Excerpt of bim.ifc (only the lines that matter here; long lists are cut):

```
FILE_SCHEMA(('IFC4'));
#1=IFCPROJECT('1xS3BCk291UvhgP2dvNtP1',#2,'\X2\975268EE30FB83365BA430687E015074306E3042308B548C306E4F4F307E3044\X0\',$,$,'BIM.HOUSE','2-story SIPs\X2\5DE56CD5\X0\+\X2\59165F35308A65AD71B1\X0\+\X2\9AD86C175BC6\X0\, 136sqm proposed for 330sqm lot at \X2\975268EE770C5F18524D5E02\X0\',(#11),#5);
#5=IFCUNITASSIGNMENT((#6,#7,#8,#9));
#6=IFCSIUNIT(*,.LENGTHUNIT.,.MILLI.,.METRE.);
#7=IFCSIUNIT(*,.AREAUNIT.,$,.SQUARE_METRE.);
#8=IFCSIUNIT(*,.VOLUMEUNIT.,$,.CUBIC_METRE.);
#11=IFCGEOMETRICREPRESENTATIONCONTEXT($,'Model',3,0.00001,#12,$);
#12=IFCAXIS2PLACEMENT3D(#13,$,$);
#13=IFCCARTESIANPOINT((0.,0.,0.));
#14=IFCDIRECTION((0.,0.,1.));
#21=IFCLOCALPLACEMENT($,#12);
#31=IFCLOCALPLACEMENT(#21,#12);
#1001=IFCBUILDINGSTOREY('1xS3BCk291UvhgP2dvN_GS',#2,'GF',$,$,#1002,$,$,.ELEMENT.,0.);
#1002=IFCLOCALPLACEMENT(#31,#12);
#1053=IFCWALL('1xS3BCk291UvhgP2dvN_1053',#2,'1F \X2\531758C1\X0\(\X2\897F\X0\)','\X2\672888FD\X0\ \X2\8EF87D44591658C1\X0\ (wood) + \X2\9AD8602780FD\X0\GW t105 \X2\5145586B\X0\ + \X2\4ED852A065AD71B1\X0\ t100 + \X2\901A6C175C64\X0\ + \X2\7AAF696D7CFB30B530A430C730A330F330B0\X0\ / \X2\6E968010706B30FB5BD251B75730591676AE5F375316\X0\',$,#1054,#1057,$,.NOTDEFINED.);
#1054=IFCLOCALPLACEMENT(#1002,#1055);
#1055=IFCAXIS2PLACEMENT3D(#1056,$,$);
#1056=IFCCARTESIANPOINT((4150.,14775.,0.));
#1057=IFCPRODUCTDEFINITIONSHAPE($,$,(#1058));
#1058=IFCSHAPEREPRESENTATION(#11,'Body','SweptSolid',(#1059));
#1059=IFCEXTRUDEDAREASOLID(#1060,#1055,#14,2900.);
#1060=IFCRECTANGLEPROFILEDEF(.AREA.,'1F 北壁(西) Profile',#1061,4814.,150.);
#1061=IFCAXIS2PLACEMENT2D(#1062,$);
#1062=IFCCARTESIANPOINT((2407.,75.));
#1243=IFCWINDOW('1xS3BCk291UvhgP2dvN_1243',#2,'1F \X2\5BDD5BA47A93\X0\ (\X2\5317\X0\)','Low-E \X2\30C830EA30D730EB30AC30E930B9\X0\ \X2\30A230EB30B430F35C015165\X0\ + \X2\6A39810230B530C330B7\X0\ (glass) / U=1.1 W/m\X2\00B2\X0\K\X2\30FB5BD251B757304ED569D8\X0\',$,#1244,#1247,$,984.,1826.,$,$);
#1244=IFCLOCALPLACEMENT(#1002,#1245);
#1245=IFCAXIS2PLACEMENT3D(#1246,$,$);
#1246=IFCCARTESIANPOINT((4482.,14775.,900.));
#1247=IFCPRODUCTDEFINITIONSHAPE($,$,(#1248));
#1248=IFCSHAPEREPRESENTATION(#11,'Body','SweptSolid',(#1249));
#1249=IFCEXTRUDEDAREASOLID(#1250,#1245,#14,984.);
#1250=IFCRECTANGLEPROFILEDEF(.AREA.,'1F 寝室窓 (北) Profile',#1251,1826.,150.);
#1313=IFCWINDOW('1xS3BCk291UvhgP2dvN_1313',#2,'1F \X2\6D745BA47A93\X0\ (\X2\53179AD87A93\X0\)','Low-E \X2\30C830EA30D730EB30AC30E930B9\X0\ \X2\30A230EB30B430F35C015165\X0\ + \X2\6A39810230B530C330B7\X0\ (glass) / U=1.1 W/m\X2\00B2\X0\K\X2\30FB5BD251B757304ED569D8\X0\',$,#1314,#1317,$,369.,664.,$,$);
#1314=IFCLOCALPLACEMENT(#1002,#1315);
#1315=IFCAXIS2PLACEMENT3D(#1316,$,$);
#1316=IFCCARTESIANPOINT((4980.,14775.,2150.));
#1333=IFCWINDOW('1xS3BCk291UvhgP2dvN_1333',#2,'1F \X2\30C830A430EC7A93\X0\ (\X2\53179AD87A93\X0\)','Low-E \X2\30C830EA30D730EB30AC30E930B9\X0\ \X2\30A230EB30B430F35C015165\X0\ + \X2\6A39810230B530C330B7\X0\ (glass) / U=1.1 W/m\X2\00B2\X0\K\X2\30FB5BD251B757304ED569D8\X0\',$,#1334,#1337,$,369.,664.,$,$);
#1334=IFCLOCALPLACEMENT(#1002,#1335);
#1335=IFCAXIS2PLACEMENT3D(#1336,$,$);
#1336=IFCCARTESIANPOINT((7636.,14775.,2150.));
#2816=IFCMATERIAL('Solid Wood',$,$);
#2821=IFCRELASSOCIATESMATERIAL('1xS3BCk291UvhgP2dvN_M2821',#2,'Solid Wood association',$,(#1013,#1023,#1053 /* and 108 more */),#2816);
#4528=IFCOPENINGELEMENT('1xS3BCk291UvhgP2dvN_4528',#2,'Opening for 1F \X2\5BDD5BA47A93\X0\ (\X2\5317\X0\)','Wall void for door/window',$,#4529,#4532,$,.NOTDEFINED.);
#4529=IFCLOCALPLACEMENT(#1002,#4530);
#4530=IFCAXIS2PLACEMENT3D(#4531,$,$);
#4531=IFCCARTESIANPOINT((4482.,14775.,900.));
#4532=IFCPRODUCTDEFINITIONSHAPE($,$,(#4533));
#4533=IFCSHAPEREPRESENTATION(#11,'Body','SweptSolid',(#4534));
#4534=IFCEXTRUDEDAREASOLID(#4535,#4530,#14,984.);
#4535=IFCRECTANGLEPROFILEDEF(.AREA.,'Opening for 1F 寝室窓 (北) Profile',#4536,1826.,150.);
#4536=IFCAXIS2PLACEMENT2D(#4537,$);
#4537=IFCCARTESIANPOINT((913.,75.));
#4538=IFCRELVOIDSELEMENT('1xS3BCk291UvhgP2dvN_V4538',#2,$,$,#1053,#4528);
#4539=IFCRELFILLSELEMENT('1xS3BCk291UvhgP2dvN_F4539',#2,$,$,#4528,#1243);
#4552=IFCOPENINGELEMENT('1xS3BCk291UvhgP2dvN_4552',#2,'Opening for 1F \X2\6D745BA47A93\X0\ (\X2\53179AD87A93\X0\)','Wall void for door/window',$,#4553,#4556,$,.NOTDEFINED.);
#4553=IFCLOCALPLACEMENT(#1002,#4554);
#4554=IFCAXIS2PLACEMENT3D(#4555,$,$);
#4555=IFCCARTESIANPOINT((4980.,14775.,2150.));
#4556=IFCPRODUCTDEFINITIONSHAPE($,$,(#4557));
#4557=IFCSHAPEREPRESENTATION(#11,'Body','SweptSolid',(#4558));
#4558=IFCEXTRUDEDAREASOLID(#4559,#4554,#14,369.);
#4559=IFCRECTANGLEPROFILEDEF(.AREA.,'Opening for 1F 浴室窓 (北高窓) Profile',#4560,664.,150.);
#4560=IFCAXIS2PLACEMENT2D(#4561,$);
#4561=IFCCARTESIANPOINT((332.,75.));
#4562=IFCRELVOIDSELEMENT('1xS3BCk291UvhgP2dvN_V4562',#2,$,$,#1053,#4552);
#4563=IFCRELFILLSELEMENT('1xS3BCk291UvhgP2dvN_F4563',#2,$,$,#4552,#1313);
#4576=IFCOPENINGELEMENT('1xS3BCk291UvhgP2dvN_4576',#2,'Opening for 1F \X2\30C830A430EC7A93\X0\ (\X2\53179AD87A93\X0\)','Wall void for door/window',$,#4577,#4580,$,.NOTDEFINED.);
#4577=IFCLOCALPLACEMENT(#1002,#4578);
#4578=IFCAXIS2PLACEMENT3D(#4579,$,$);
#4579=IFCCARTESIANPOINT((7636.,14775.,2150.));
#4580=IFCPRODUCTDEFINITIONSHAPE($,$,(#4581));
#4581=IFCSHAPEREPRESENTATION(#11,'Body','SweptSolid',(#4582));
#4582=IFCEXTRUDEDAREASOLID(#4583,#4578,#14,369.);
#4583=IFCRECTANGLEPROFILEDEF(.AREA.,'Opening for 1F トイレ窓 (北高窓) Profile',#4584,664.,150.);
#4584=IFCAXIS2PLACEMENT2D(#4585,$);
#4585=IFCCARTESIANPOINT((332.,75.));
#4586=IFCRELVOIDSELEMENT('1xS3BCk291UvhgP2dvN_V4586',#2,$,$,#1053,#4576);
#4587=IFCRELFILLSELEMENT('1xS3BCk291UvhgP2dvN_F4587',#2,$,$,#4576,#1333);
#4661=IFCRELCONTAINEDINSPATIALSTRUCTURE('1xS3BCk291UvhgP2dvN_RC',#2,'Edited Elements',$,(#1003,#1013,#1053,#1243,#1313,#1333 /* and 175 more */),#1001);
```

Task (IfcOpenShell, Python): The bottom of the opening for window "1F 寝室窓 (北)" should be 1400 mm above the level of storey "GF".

```python
import numpy as np
import ifcopenshell
import ifcopenshell.api.geometry
import ifcopenshell.geom
import ifcopenshell.util.element
import ifcopenshell.util.placement
import ifcopenshell.util.shape
import ifcopenshell.util.unit

model = ifcopenshell.open("bim.ifc")
unit_scale = ifcopenshell.util.unit.calculate_unit_scale(model)

window = model.by_id(1243)
opening = window.FillsVoids[0].RelatingOpeningElement
storey = ifcopenshell.util.element.get_container(window, ifc_class="IfcBuildingStorey")
level = ifcopenshell.util.placement.get_local_placement(storey.ObjectPlacement)[2, 3]

# The opening's origin need not be at the sill, so measure its lowest point.
shape = ifcopenshell.geom.create_shape(ifcopenshell.geom.settings(), opening)
bottom = ifcopenshell.util.shape.get_shape_bottom_elevation(shape, shape.geometry) / unit_scale
dz = level + 1400.0 - bottom

shift = np.array([0.0, 0.0, dz])
# The window is not placed relative to its opening, so move both.
for product in (opening, window):
    matrix = ifcopenshell.util.placement.get_local_placement(product.ObjectPlacement)
    matrix[:3, 3] += shift
    ifcopenshell.api.geometry.edit_object_placement(model, product=product, matrix=matrix, is_si=False)

print(f"moved by {dz * unit_scale:+.3f} m")

model.write("bim-out.ifc")
```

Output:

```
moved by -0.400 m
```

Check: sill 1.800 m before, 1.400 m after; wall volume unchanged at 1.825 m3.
